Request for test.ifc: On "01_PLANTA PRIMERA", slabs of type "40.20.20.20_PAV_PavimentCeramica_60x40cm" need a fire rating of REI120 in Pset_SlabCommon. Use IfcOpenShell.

First a look at what the model holds.

```python
import ifcopenshell
import ifcopenshell.util.element

model = ifcopenshell.open("test.ifc")
print(model.schema)
storey = next(s for s in model.by_type("IfcBuildingStorey") if s.Name == "01_PLANTA PRIMERA")
slabs = [e for e in ifcopenshell.util.element.get_decomposition(storey) if e.is_a("IfcSlab")]
seen = {}
for e in slabs:
    element_type = ifcopenshell.util.element.get_type(e)
    key = (element_type.Name if element_type != e and element_type else None, ifcopenshell.util.element.get_pset(e, "Pset_SlabCommon", "FireRating"))
    seen[key] = seen.get(key, 0) + 1
for (name, value), count in sorted(seen.items(), key=str):
    print(count, "x", name, "|", value)
```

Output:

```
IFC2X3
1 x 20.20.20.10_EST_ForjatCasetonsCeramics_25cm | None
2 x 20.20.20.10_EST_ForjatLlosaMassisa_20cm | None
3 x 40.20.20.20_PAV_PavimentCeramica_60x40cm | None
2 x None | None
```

```python
import ifcopenshell
import ifcopenshell.api.pset
import ifcopenshell.util.element

model = ifcopenshell.open("test.ifc")

storey = next(s for s in model.by_type("IfcBuildingStorey") if s.Name == "01_PLANTA PRIMERA")
slabs = [e for e in ifcopenshell.util.element.get_decomposition(storey) if e.is_a("IfcSlab")]

count = 0
for e in slabs:
    element_type = ifcopenshell.util.element.get_type(e)
    if element_type in (None, e) or element_type.Name != "40.20.20.20_PAV_PavimentCeramica_60x40cm":
        continue
    # add_pset returns the element's existing set when there is one.
    pset = ifcopenshell.api.pset.add_pset(model, product=e, name="Pset_SlabCommon")
    ifcopenshell.api.pset.edit_pset(model, pset=pset, properties={"FireRating": "REI120"})
    count += 1

print(count, "slabs updated")

model.write("test_rev.ifc")
```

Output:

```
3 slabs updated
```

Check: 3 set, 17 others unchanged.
